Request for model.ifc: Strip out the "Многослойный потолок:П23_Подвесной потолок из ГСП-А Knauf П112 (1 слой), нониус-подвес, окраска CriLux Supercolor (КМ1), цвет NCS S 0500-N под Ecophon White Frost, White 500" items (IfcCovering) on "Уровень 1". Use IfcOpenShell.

First a look at what the model holds.

```python
import ifcopenshell
import ifcopenshell.util.element

model = ifcopenshell.open("model.ifc")
print(model.schema)
storey = next(s for s in model.by_type("IfcBuildingStorey") if s.Name == "Уровень 1")
coverings = [e for e in ifcopenshell.util.element.get_decomposition(storey) if e.is_a("IfcCovering")]
seen = {}
for e in coverings:
    element_type = ifcopenshell.util.element.get_type(e)
    name = element_type.Name if element_type not in (None, e) else None
    seen[name] = seen.get(name, 0) + 1
for name, count in sorted(seen.items(), key=str):
    print(count, "x", name)
```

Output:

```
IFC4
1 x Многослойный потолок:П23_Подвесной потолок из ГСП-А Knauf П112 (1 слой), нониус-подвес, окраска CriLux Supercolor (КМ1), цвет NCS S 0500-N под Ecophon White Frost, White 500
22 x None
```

```python
import ifcopenshell
import ifcopenshell.api.root
import ifcopenshell.util.element

model = ifcopenshell.open("model.ifc")

storey = next(s for s in model.by_type("IfcBuildingStorey") if s.Name == "Уровень 1")
coverings = [e for e in ifcopenshell.util.element.get_decomposition(storey) if e.is_a("IfcCovering")]
targets = [e for e in coverings if (t := ifcopenshell.util.element.get_type(e)) not in (None, e) and t.Name == "Многослойный потолок:П23_Подвесной потолок из ГСП-А Knauf П112 (1 слой), нониус-подвес, окраска CriLux Supercolor (КМ1), цвет NCS S 0500-N под Ecophon White Frost, White 500"]

for e in targets:
    ifcopenshell.api.root.remove_product(model, product=e)
print(len(targets), "removed")

model.write("model_rev.ifc")
```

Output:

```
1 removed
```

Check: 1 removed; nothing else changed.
